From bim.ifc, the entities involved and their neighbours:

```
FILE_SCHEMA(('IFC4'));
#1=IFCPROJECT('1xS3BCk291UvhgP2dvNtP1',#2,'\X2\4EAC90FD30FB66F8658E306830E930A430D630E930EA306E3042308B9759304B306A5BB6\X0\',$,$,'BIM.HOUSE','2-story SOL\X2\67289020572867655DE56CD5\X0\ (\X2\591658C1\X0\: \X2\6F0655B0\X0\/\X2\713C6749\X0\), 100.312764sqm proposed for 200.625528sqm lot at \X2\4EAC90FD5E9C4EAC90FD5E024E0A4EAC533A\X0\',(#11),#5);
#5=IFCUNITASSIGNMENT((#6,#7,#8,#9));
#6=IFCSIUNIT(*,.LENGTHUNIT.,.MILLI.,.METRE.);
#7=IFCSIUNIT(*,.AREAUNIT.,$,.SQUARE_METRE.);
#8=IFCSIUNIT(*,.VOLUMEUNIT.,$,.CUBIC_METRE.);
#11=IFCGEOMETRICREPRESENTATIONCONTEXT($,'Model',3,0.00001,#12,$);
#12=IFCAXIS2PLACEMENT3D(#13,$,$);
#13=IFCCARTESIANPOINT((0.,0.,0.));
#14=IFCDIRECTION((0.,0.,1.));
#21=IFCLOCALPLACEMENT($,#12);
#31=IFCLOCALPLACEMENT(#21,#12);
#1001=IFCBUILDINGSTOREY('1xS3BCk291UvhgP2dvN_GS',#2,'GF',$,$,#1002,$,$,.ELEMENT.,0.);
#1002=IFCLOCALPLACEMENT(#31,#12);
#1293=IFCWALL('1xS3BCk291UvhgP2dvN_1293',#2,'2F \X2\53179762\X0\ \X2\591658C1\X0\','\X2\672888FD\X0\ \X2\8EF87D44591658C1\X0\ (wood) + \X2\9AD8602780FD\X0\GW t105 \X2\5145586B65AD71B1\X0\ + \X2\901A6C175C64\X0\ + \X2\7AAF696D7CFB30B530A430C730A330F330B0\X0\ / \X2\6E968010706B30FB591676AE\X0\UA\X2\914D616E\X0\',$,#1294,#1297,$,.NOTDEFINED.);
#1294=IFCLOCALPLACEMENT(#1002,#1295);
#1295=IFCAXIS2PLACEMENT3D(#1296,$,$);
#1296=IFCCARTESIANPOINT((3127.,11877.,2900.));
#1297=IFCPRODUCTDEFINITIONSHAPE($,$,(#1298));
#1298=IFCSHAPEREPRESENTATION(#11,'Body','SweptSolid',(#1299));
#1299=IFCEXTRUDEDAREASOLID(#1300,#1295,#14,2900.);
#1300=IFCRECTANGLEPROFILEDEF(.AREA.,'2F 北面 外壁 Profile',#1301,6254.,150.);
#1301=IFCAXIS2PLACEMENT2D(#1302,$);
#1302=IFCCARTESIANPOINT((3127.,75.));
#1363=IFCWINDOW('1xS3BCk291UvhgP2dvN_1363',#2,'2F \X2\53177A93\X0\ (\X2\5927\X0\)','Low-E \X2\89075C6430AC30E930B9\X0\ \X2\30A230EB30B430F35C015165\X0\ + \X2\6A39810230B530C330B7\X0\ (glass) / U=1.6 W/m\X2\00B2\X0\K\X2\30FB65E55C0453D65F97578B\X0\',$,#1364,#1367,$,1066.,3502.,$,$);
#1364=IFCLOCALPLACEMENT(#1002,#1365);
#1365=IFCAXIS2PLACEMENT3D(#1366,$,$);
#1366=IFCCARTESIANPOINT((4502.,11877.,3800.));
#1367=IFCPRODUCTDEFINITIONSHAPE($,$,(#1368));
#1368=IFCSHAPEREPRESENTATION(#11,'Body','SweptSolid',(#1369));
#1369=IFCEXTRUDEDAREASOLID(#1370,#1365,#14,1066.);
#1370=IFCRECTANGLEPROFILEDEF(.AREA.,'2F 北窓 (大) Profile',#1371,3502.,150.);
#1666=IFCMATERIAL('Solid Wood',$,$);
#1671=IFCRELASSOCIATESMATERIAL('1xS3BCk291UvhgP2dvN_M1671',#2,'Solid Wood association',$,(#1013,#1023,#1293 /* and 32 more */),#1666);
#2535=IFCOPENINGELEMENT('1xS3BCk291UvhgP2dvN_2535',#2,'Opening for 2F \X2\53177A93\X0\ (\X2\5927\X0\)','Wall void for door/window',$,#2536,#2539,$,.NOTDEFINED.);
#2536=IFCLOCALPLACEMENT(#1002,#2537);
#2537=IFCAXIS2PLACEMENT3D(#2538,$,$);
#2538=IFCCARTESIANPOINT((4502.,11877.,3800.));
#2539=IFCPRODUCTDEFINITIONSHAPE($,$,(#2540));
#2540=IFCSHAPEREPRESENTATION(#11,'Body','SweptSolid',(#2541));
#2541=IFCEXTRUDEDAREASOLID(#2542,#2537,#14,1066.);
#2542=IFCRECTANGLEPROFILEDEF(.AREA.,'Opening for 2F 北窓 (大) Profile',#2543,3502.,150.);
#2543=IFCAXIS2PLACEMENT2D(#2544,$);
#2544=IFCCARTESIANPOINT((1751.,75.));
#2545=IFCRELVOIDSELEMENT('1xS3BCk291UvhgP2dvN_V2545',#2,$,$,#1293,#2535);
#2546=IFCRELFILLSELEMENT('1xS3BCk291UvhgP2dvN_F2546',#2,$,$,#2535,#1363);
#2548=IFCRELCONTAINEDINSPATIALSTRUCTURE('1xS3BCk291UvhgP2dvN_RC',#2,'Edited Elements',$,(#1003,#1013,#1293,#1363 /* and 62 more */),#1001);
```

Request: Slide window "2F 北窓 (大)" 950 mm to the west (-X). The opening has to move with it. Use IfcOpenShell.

```python
import ifcopenshell
import ifcopenshell.api.geometry
import ifcopenshell.util.placement
import ifcopenshell.util.unit

model = ifcopenshell.open("bim.ifc")
unit_scale = ifcopenshell.util.unit.calculate_unit_scale(model)

window = model.by_id(1363)
opening = window.FillsVoids[0].RelatingOpeningElement
wall = opening.VoidsElements[0].RelatingBuildingElement

wall_matrix = ifcopenshell.util.placement.get_local_placement(wall.ObjectPlacement)
shift = wall_matrix[:3, 0] * -0.95 / unit_scale
before = ifcopenshell.util.placement.get_local_placement(window.ObjectPlacement)[:3, 3].copy()

# The window is not placed relative to its opening, so move both.
for product in (opening, window):
    matrix = ifcopenshell.util.placement.get_local_placement(product.ObjectPlacement)
    matrix[:3, 3] += shift
    ifcopenshell.api.geometry.edit_object_placement(model, product=product, matrix=matrix, is_si=False)

after = ifcopenshell.util.placement.get_local_placement(window.ObjectPlacement)[:3, 3]
print("window moved by", (after - before).round(3) + 0.0)

model.write("bim_v2.ifc")
```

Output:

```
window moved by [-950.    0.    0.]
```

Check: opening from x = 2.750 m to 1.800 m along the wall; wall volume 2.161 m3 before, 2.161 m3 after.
